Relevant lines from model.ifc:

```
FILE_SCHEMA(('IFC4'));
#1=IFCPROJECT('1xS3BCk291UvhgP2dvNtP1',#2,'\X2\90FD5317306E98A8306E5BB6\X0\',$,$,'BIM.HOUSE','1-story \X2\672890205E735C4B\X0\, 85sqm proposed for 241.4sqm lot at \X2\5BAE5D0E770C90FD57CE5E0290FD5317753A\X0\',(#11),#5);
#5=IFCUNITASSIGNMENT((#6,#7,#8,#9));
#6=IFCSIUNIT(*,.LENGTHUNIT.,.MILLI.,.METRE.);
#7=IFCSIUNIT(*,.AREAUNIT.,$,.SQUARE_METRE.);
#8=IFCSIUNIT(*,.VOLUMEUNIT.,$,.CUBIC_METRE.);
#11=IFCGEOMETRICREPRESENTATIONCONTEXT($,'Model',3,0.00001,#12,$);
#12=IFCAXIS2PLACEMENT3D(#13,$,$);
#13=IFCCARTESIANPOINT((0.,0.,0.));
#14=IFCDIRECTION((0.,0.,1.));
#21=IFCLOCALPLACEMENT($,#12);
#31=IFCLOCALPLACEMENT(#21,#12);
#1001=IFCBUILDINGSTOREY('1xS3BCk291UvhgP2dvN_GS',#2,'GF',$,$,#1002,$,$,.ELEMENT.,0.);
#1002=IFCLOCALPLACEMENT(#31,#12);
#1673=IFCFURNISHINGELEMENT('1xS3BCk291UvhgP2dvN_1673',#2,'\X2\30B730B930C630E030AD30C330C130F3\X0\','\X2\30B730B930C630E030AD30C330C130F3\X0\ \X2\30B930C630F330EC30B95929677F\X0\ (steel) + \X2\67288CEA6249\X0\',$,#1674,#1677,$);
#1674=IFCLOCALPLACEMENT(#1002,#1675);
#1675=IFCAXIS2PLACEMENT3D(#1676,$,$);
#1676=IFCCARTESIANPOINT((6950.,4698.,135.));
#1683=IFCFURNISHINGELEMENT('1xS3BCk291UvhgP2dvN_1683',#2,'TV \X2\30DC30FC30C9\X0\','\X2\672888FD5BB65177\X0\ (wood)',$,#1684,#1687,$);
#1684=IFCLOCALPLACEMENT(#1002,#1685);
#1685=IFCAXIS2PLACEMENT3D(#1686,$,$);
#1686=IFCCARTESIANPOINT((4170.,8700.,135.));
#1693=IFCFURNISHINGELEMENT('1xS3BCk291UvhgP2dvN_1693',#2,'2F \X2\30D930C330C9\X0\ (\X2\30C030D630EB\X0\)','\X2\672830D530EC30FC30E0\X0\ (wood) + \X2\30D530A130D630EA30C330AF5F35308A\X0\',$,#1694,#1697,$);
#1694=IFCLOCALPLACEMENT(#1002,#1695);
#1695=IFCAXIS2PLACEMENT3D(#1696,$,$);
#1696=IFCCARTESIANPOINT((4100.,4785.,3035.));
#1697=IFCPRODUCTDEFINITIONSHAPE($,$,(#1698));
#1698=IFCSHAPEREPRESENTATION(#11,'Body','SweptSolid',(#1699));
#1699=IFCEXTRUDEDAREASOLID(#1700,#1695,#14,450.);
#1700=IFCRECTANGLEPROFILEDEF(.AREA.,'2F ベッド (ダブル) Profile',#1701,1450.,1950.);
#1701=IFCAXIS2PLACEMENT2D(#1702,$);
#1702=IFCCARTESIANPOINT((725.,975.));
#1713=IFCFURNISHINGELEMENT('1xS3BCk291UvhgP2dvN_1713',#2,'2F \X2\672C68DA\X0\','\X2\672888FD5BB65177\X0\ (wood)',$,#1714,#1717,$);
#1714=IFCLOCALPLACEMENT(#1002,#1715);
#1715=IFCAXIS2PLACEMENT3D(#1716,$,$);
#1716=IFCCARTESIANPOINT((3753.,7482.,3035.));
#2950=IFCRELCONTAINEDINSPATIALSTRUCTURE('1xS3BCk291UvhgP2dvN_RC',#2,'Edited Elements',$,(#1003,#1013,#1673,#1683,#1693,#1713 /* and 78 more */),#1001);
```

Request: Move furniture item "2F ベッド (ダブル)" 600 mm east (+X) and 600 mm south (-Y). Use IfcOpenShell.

```python
import ifcopenshell
import ifcopenshell.api.geometry
import ifcopenshell.util.placement
import ifcopenshell.util.unit

model = ifcopenshell.open("model.ifc")
unit_scale = ifcopenshell.util.unit.calculate_unit_scale(model)

item = model.by_guid("1xS3BCk291UvhgP2dvN_1693")
matrix = ifcopenshell.util.placement.get_local_placement(item.ObjectPlacement)
matrix[0, 3] += 0.6 / unit_scale
matrix[1, 3] -= 0.6 / unit_scale
ifcopenshell.api.geometry.edit_object_placement(model, product=item, matrix=matrix, is_si=False)

print(ifcopenshell.util.placement.get_local_placement(item.ObjectPlacement).round(3) + 0.0)

model.write("model_updated.ifc")
```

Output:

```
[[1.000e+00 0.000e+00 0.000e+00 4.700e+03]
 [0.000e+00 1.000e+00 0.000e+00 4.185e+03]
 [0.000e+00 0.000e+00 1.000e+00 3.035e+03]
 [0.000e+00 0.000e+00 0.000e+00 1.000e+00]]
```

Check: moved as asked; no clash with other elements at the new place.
